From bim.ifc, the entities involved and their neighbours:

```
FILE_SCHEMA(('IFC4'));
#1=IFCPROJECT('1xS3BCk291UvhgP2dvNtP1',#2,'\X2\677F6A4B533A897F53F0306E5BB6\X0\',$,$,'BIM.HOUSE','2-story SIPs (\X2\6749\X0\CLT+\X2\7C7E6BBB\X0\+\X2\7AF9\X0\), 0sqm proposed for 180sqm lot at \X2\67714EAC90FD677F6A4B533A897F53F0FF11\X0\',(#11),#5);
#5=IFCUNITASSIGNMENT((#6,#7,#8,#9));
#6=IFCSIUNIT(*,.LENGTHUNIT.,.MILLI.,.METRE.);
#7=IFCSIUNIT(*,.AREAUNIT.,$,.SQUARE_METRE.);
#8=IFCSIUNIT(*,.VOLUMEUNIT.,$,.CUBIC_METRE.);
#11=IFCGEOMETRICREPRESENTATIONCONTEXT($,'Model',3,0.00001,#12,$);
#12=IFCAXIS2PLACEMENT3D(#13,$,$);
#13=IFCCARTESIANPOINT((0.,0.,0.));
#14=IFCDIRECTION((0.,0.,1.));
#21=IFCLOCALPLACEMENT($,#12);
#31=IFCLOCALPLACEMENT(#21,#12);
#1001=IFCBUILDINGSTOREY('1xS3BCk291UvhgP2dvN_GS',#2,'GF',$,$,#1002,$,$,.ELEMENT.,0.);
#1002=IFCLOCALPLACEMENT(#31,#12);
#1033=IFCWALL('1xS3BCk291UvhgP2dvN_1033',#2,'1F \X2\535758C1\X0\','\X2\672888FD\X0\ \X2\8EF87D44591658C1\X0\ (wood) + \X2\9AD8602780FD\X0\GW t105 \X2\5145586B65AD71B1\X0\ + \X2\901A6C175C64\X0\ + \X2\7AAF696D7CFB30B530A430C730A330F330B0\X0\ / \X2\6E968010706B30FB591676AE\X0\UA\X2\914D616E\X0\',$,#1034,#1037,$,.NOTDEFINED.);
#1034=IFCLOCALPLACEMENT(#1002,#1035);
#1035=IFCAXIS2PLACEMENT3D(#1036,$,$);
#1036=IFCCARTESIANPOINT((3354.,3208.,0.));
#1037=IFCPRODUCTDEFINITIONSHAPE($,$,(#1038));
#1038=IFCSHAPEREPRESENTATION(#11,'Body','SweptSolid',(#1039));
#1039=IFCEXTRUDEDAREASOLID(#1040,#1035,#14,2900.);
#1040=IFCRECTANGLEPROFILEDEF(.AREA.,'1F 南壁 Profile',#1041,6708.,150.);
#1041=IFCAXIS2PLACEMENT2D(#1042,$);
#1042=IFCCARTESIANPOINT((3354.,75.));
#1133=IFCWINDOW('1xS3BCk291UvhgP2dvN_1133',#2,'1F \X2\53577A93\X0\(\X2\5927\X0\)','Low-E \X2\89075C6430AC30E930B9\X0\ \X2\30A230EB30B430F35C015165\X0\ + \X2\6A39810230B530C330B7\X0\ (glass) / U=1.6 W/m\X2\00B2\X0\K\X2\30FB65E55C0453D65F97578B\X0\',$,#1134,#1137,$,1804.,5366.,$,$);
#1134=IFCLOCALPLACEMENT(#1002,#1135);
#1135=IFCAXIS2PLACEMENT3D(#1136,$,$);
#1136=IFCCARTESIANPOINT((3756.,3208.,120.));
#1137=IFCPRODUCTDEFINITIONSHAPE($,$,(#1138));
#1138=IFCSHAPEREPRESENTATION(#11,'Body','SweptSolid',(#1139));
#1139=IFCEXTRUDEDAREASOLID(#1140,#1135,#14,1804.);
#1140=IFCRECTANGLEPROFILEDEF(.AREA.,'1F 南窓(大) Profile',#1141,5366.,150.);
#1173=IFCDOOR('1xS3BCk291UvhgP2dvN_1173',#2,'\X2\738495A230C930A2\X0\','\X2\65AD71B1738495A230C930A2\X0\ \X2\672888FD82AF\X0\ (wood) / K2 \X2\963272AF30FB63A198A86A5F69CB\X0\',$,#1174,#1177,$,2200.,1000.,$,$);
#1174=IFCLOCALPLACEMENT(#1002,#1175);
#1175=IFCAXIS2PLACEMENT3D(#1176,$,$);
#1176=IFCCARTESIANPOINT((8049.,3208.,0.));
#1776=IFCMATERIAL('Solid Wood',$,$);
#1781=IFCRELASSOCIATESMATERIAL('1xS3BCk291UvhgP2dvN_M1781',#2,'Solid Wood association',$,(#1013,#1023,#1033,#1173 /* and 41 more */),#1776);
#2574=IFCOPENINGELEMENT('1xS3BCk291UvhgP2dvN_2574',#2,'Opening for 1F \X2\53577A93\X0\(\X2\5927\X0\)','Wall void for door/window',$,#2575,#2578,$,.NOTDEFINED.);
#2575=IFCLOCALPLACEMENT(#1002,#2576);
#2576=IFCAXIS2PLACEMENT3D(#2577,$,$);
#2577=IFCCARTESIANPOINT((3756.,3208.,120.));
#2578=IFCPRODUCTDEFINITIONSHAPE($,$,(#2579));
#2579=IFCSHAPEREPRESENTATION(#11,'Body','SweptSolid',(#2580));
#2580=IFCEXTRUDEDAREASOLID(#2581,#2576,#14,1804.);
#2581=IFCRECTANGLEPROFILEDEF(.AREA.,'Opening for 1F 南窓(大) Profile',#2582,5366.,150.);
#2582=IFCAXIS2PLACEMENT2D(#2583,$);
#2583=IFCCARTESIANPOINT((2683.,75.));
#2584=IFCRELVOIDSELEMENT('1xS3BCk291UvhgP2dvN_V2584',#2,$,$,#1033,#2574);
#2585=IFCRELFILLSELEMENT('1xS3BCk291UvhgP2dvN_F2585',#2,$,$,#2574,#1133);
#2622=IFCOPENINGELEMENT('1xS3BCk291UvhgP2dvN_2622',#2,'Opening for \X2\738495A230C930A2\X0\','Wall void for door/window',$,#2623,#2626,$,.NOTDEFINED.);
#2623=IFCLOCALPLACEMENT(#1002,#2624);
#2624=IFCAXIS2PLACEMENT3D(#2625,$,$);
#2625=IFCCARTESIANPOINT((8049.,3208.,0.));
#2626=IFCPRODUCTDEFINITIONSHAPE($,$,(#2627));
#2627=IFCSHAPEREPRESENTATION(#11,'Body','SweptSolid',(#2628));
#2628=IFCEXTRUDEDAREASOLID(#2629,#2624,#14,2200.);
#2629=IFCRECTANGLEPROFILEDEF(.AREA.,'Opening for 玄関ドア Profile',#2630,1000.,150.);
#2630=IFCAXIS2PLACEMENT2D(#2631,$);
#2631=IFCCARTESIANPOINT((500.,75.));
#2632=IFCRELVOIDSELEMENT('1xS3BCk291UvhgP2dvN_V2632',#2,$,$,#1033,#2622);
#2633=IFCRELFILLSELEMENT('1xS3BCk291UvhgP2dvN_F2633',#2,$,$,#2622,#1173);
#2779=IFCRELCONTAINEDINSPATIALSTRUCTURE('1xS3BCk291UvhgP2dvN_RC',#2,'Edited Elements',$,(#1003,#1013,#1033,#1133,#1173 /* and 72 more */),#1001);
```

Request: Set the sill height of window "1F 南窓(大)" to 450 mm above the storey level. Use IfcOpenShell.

```python
import numpy as np
import ifcopenshell
import ifcopenshell.api.geometry
import ifcopenshell.geom
import ifcopenshell.util.element
import ifcopenshell.util.placement
import ifcopenshell.util.shape
import ifcopenshell.util.unit

model = ifcopenshell.open("bim.ifc")
unit_scale = ifcopenshell.util.unit.calculate_unit_scale(model)

window = model.by_guid("1xS3BCk291UvhgP2dvN_1133")
opening = window.FillsVoids[0].RelatingOpeningElement
storey = ifcopenshell.util.element.get_container(window, ifc_class="IfcBuildingStorey")
level = ifcopenshell.util.placement.get_local_placement(storey.ObjectPlacement)[2, 3]

# The opening's origin need not be at the sill, so measure its lowest point.
shape = ifcopenshell.geom.create_shape(ifcopenshell.geom.settings(), opening)
bottom = ifcopenshell.util.shape.get_shape_bottom_elevation(shape, shape.geometry) / unit_scale
dz = level + 0.45 / unit_scale - bottom

shift = np.array([0.0, 0.0, dz])
# The window is not placed relative to its opening, so move both.
for product in (opening, window):
    matrix = ifcopenshell.util.placement.get_local_placement(product.ObjectPlacement)
    matrix[:3, 3] += shift
    ifcopenshell.api.geometry.edit_object_placement(model, product=product, matrix=matrix, is_si=False)

print(f"moved by {dz * unit_scale:+.3f} m")

model.write("bim_updated.ifc")
```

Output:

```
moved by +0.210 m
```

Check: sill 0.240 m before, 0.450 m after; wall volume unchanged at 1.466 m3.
